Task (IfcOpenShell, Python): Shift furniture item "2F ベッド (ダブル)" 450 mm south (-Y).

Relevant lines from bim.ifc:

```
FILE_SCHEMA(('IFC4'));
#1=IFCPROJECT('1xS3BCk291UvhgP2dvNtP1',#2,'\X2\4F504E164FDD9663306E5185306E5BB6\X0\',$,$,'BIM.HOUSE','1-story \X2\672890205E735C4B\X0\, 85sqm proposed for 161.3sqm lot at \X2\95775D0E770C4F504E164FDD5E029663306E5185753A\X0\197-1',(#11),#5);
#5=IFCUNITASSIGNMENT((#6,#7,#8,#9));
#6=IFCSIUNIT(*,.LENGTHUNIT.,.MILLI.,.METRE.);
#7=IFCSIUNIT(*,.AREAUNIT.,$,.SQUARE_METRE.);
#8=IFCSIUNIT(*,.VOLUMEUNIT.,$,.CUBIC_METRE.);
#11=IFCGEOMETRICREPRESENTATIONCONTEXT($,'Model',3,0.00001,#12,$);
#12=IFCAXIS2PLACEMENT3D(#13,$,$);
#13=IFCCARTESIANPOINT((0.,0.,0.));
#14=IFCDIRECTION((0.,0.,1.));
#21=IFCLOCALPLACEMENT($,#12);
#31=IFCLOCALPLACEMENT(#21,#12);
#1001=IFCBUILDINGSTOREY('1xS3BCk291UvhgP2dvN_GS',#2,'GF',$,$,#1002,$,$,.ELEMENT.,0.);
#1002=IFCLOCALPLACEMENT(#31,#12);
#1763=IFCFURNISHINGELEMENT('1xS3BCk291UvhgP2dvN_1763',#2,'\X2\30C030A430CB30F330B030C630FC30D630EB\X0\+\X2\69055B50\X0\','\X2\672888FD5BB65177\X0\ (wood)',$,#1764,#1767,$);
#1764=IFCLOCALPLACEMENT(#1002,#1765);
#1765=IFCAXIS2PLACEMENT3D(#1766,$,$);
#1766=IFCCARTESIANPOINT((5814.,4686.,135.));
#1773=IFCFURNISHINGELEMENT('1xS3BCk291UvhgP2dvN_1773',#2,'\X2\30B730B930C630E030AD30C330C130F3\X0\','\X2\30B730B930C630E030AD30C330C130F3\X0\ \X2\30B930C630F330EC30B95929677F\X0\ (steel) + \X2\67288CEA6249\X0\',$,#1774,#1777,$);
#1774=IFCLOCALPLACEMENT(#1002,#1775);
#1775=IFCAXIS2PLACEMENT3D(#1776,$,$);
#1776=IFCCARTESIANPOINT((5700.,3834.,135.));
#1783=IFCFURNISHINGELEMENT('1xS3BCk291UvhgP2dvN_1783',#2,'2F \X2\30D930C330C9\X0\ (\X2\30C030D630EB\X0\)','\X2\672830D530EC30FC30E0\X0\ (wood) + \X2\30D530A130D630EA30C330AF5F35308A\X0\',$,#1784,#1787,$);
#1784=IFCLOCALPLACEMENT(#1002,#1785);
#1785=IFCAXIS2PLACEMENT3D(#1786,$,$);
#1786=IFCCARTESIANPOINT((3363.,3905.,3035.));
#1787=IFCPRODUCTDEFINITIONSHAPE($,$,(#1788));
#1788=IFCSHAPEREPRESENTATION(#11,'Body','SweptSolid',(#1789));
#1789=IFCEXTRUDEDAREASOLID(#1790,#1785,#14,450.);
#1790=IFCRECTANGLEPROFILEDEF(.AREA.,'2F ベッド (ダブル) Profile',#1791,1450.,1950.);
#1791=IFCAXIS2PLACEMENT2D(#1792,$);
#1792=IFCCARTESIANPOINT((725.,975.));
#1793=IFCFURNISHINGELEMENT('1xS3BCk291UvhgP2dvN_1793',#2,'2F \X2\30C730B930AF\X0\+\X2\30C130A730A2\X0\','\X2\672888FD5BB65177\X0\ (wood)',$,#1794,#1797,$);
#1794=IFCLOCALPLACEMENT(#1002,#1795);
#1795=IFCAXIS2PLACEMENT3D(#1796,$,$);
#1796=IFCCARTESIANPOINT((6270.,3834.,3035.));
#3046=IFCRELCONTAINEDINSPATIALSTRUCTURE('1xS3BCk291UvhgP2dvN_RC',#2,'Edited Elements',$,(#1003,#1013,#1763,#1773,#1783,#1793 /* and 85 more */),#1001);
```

```python
import ifcopenshell
import ifcopenshell.api.geometry
import ifcopenshell.util.placement

model = ifcopenshell.open("bim.ifc")

item = model.by_id(1783)
matrix = ifcopenshell.util.placement.get_local_placement(item.ObjectPlacement)
matrix[1, 3] -= 450.0
ifcopenshell.api.geometry.edit_object_placement(model, product=item, matrix=matrix, is_si=False)

print(ifcopenshell.util.placement.get_local_placement(item.ObjectPlacement).round(3) + 0.0)

model.write("bim_edited.ifc")
```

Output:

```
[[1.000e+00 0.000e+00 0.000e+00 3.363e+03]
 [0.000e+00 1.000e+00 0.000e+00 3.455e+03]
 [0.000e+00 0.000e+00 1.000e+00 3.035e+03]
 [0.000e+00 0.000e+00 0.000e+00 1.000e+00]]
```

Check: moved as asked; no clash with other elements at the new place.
